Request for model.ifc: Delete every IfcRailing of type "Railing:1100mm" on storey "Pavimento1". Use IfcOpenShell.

First a look at what the model holds.

```python
import ifcopenshell
import ifcopenshell.util.element

model = ifcopenshell.open("model.ifc")
print(model.schema)
storey = next(s for s in model.by_type("IfcBuildingStorey") if s.Name == "Pavimento1")
railings = [e for e in ifcopenshell.util.element.get_decomposition(storey) if e.is_a("IfcRailing")]
seen = {}
for e in railings:
    element_type = ifcopenshell.util.element.get_type(e)
    name = element_type.Name if element_type not in (None, e) else None
    seen[name] = seen.get(name, 0) + 1
for name, count in sorted(seen.items(), key=str):
    print(count, "x", name)
```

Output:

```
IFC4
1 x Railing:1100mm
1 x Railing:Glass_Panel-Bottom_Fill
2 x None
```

```python
import ifcopenshell
import ifcopenshell.api.root
import ifcopenshell.util.element

model = ifcopenshell.open("model.ifc")

storey = next(s for s in model.by_type("IfcBuildingStorey") if s.Name == "Pavimento1")
railings = [e for e in ifcopenshell.util.element.get_decomposition(storey) if e.is_a("IfcRailing")]
targets = [e for e in railings if (t := ifcopenshell.util.element.get_type(e)) not in (None, e) and t.Name == "Railing:1100mm"]

for e in targets:
    ifcopenshell.api.root.remove_product(model, product=e)
print(len(targets), "removed")

model.write("model_edited.ifc")
```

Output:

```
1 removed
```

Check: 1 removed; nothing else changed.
